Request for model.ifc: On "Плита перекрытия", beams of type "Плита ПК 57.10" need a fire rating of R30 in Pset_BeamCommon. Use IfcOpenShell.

First a look at what the model holds.

```python
import ifcopenshell
import ifcopenshell.util.element

model = ifcopenshell.open("model.ifc")
print(model.schema)
storey = next(s for s in model.by_type("IfcBuildingStorey") if s.Name == "Плита перекрытия")
beams = [e for e in ifcopenshell.util.element.get_decomposition(storey) if e.is_a("IfcBeam")]
seen = {}
for e in beams:
    element_type = ifcopenshell.util.element.get_type(e)
    key = (element_type.Name if element_type != e and element_type else None, ifcopenshell.util.element.get_pset(e, "Pset_BeamCommon", "FireRating"))
    seen[key] = seen.get(key, 0) + 1
for (name, value), count in sorted(seen.items(), key=str):
    print(count, "x", name, "|", value)
```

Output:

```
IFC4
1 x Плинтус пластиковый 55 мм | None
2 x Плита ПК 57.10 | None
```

```python
import ifcopenshell
import ifcopenshell.api.pset
import ifcopenshell.util.element

model = ifcopenshell.open("model.ifc")

storey = next(s for s in model.by_type("IfcBuildingStorey") if s.Name == "Плита перекрытия")
beams = [e for e in ifcopenshell.util.element.get_decomposition(storey) if e.is_a("IfcBeam")]

count = 0
for e in beams:
    element_type = ifcopenshell.util.element.get_type(e)
    if element_type in (None, e) or element_type.Name != "Плита ПК 57.10":
        continue
    # add_pset returns the element's existing set when there is one.
    pset = ifcopenshell.api.pset.add_pset(model, product=e, name="Pset_BeamCommon")
    ifcopenshell.api.pset.edit_pset(model, pset=pset, properties={"FireRating": "R30"})
    count += 1

print(count, "beams updated")

model.write("model-out.ifc")
```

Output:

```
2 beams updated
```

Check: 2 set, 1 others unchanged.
